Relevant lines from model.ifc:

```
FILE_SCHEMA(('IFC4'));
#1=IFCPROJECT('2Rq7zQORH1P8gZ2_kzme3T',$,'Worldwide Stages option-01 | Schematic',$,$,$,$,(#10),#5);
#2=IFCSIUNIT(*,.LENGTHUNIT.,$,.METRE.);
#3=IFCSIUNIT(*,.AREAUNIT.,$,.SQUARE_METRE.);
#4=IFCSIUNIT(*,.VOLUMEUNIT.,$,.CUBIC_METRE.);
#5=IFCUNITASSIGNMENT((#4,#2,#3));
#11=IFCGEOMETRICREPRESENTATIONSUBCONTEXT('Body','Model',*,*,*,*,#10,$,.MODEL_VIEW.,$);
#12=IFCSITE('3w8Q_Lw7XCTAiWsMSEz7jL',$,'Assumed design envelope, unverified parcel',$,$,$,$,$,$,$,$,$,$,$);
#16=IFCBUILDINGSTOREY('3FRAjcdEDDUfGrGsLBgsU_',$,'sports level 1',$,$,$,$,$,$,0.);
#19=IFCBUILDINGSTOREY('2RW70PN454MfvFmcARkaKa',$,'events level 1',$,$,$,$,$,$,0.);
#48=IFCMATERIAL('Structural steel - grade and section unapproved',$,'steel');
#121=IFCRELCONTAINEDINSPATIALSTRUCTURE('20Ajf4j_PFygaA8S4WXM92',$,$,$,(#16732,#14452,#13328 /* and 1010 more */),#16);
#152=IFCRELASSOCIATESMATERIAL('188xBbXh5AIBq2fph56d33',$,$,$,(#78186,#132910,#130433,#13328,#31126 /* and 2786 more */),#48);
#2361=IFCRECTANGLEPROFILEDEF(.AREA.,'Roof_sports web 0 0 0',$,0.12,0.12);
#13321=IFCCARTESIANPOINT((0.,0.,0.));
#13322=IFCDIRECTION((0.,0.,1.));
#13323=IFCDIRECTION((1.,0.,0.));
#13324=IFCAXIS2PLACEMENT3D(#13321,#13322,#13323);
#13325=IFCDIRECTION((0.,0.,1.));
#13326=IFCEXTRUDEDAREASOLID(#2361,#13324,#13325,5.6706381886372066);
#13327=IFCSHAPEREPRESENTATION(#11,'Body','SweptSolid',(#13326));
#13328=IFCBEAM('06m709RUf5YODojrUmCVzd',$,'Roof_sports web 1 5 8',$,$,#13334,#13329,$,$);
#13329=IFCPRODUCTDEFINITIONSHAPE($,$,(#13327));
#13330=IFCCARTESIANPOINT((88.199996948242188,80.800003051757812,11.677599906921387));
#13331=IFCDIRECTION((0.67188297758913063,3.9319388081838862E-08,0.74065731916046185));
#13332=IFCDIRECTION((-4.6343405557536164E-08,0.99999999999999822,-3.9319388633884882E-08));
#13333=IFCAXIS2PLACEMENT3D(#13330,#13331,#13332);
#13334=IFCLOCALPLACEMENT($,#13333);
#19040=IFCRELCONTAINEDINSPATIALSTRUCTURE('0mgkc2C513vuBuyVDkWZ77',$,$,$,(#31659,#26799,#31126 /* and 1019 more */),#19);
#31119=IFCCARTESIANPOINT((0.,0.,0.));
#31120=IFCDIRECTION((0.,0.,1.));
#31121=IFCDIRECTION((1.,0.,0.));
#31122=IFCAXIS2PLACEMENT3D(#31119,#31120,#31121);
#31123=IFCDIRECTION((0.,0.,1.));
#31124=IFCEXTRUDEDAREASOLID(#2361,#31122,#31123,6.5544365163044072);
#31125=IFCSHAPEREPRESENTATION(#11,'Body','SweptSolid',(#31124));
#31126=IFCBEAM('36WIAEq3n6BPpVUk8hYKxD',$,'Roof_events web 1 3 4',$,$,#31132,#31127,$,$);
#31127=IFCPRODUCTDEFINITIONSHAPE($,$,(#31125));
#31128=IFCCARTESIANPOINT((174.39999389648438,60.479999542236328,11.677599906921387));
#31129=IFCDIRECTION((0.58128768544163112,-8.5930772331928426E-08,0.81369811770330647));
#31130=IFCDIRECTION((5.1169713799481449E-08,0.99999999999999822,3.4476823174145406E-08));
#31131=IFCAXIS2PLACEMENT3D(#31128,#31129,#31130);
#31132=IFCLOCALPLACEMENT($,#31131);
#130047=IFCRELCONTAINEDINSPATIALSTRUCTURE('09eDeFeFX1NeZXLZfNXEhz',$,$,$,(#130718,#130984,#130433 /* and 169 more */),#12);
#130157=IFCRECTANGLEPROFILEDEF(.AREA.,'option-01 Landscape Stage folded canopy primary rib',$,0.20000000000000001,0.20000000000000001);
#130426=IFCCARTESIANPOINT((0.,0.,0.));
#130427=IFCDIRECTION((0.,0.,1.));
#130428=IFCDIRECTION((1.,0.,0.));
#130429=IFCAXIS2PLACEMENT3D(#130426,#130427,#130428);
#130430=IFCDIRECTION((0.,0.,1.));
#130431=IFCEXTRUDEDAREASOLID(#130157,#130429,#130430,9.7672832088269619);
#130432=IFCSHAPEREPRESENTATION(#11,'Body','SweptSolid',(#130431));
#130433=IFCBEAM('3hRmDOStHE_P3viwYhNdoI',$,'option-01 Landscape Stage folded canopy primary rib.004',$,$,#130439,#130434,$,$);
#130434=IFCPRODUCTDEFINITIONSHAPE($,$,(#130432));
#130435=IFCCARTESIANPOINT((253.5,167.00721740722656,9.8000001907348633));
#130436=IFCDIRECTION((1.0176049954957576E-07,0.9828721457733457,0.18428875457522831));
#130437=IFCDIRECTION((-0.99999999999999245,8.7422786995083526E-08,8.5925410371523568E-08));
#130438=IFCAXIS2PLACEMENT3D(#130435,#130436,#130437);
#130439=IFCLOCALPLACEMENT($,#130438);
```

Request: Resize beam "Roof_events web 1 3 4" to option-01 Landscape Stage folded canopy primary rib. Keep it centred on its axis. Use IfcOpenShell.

```python
import ifcopenshell
import ifcopenshell.util.element
import ifcopenshell.util.representation

model = ifcopenshell.open("model.ifc")

member = model.by_guid("36WIAEq3n6BPpVUk8hYKxD")
source = next(p for p in model.by_type("IfcRectangleProfileDef") if p.ProfileName == "option-01 Landscape Stage folded canopy primary rib")

body = ifcopenshell.util.representation.get_representation(member, "Model", "Body")
solid = body.Items[0]
old_profile = solid.SweptArea

# Copy the section's sizes but keep this member's own profile position.
profile = ifcopenshell.util.element.copy(model, source)
profile.Position = old_profile.Position
solid.SweptArea = profile
if not model.get_total_inverses(old_profile):
    ifcopenshell.util.element.remove_deep2(model, old_profile)

print(solid.SweptArea)

model.write("model_rev.ifc")
```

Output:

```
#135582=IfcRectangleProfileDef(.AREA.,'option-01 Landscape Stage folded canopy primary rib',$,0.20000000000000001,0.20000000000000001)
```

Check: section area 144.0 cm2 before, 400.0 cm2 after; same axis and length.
